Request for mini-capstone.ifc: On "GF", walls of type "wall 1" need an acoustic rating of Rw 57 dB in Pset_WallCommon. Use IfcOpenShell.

First a look at what the model holds.

```python
import ifcopenshell
import ifcopenshell.util.element

model = ifcopenshell.open("mini-capstone.ifc")
print(model.schema)
storey = next(s for s in model.by_type("IfcBuildingStorey") if s.Name == "GF")
walls = [e for e in ifcopenshell.util.element.get_decomposition(storey) if e.is_a("IfcWall")]
seen = {}
for e in walls:
    element_type = ifcopenshell.util.element.get_type(e)
    key = (element_type.Name if element_type != e and element_type else None, ifcopenshell.util.element.get_pset(e, "Pset_WallCommon", "AcousticRating"))
    seen[key] = seen.get(key, 0) + 1
for (name, value), count in sorted(seen.items(), key=str):
    print(count, "x", name, "|", value)
```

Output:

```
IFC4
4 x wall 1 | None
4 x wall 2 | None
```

```python
import ifcopenshell
import ifcopenshell.api.pset
import ifcopenshell.util.element

model = ifcopenshell.open("mini-capstone.ifc")

storey = next(s for s in model.by_type("IfcBuildingStorey") if s.Name == "GF")
walls = [e for e in ifcopenshell.util.element.get_decomposition(storey) if e.is_a("IfcWall")]

count = 0
for e in walls:
    element_type = ifcopenshell.util.element.get_type(e)
    if element_type in (None, e) or element_type.Name != "wall 1":
        continue
    # add_pset returns the element's existing set when there is one.
    pset = ifcopenshell.api.pset.add_pset(model, product=e, name="Pset_WallCommon")
    ifcopenshell.api.pset.edit_pset(model, pset=pset, properties={"AcousticRating": "Rw 57 dB"})
    count += 1

print(count, "walls updated")

model.write("mini-capstone_updated.ifc")
```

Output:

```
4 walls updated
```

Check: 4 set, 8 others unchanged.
